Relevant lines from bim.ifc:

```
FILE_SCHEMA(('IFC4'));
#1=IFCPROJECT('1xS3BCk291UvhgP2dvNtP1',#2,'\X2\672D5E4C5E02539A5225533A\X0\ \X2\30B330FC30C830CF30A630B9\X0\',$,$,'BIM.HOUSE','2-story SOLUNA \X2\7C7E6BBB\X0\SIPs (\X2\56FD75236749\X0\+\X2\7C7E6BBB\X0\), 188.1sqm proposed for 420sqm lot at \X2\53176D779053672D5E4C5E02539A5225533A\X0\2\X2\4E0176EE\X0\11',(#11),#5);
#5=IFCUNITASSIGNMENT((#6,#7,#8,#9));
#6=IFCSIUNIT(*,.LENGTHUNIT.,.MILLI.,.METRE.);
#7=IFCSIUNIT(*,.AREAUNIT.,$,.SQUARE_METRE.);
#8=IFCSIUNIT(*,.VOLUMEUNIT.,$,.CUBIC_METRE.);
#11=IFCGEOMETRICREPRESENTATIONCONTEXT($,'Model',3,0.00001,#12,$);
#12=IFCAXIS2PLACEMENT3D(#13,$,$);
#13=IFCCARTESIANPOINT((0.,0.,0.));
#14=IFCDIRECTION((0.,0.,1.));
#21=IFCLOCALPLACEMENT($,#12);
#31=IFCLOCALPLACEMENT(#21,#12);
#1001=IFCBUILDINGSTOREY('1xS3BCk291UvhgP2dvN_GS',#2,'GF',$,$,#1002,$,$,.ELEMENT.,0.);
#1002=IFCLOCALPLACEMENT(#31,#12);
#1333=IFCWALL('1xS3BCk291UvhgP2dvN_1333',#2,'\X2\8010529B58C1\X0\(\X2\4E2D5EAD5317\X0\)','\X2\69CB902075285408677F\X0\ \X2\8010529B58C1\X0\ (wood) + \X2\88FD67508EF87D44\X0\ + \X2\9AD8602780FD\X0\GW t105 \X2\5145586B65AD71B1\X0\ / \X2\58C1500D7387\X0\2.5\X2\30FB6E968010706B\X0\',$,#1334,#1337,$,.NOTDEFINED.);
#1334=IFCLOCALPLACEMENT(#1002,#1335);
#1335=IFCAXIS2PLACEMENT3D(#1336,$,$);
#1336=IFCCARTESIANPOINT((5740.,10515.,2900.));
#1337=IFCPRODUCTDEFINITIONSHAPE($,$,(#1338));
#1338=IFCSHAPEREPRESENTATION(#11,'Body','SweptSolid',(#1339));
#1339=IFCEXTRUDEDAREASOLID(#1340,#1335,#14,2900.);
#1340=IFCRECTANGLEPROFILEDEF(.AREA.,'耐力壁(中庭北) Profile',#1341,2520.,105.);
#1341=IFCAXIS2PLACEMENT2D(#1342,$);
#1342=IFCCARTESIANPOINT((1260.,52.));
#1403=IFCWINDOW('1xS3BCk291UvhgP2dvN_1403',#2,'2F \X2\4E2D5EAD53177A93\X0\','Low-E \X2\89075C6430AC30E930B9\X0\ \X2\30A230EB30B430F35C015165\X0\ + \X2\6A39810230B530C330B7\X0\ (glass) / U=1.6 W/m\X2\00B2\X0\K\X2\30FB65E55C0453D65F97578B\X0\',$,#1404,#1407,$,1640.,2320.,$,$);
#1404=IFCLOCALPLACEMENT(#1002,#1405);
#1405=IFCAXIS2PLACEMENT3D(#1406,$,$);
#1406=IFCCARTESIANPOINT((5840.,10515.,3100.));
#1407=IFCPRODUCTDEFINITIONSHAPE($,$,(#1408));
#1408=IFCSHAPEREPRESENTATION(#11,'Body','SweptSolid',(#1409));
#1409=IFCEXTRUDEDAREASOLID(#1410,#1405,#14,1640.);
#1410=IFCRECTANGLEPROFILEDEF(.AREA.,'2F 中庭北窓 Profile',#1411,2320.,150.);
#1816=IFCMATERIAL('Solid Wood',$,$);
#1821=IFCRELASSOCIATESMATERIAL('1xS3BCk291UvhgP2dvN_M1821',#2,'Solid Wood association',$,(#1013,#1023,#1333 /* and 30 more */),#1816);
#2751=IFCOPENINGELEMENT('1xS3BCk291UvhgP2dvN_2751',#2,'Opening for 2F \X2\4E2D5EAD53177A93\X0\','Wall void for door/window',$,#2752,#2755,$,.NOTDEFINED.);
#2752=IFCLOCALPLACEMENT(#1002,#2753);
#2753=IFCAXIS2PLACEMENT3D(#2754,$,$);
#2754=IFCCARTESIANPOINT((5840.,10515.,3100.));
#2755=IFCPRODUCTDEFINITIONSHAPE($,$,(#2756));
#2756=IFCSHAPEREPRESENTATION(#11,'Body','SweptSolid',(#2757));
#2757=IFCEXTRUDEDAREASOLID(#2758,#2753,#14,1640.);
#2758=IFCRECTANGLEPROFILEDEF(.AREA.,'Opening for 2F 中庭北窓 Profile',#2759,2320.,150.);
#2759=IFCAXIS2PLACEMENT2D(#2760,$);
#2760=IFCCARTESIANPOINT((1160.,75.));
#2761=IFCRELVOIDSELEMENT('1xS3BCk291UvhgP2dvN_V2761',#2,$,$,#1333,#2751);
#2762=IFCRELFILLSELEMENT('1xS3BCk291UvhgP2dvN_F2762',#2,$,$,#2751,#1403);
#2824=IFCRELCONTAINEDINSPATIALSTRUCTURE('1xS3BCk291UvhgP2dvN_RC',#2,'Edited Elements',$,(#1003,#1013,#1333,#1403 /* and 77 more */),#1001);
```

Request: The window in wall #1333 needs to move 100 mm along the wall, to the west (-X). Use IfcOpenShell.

```python
import ifcopenshell
import ifcopenshell.api.geometry
import ifcopenshell.util.placement
import ifcopenshell.util.unit

model = ifcopenshell.open("bim.ifc")
unit_scale = ifcopenshell.util.unit.calculate_unit_scale(model)

window = model.by_guid("1xS3BCk291UvhgP2dvN_1403")
opening = window.FillsVoids[0].RelatingOpeningElement
wall = opening.VoidsElements[0].RelatingBuildingElement

wall_matrix = ifcopenshell.util.placement.get_local_placement(wall.ObjectPlacement)
shift = wall_matrix[:3, 0] * -0.1 / unit_scale
before = ifcopenshell.util.placement.get_local_placement(window.ObjectPlacement)[:3, 3].copy()

# The window is not placed relative to its opening, so move both.
for product in (opening, window):
    matrix = ifcopenshell.util.placement.get_local_placement(product.ObjectPlacement)
    matrix[:3, 3] += shift
    ifcopenshell.api.geometry.edit_object_placement(model, product=product, matrix=matrix, is_si=False)

after = ifcopenshell.util.placement.get_local_placement(window.ObjectPlacement)[:3, 3]
print("window moved by", (after - before).round(3) + 0.0)

model.write("bim_v2.ifc")
```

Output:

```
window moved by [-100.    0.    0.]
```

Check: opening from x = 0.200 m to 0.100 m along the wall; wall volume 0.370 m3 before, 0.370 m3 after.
